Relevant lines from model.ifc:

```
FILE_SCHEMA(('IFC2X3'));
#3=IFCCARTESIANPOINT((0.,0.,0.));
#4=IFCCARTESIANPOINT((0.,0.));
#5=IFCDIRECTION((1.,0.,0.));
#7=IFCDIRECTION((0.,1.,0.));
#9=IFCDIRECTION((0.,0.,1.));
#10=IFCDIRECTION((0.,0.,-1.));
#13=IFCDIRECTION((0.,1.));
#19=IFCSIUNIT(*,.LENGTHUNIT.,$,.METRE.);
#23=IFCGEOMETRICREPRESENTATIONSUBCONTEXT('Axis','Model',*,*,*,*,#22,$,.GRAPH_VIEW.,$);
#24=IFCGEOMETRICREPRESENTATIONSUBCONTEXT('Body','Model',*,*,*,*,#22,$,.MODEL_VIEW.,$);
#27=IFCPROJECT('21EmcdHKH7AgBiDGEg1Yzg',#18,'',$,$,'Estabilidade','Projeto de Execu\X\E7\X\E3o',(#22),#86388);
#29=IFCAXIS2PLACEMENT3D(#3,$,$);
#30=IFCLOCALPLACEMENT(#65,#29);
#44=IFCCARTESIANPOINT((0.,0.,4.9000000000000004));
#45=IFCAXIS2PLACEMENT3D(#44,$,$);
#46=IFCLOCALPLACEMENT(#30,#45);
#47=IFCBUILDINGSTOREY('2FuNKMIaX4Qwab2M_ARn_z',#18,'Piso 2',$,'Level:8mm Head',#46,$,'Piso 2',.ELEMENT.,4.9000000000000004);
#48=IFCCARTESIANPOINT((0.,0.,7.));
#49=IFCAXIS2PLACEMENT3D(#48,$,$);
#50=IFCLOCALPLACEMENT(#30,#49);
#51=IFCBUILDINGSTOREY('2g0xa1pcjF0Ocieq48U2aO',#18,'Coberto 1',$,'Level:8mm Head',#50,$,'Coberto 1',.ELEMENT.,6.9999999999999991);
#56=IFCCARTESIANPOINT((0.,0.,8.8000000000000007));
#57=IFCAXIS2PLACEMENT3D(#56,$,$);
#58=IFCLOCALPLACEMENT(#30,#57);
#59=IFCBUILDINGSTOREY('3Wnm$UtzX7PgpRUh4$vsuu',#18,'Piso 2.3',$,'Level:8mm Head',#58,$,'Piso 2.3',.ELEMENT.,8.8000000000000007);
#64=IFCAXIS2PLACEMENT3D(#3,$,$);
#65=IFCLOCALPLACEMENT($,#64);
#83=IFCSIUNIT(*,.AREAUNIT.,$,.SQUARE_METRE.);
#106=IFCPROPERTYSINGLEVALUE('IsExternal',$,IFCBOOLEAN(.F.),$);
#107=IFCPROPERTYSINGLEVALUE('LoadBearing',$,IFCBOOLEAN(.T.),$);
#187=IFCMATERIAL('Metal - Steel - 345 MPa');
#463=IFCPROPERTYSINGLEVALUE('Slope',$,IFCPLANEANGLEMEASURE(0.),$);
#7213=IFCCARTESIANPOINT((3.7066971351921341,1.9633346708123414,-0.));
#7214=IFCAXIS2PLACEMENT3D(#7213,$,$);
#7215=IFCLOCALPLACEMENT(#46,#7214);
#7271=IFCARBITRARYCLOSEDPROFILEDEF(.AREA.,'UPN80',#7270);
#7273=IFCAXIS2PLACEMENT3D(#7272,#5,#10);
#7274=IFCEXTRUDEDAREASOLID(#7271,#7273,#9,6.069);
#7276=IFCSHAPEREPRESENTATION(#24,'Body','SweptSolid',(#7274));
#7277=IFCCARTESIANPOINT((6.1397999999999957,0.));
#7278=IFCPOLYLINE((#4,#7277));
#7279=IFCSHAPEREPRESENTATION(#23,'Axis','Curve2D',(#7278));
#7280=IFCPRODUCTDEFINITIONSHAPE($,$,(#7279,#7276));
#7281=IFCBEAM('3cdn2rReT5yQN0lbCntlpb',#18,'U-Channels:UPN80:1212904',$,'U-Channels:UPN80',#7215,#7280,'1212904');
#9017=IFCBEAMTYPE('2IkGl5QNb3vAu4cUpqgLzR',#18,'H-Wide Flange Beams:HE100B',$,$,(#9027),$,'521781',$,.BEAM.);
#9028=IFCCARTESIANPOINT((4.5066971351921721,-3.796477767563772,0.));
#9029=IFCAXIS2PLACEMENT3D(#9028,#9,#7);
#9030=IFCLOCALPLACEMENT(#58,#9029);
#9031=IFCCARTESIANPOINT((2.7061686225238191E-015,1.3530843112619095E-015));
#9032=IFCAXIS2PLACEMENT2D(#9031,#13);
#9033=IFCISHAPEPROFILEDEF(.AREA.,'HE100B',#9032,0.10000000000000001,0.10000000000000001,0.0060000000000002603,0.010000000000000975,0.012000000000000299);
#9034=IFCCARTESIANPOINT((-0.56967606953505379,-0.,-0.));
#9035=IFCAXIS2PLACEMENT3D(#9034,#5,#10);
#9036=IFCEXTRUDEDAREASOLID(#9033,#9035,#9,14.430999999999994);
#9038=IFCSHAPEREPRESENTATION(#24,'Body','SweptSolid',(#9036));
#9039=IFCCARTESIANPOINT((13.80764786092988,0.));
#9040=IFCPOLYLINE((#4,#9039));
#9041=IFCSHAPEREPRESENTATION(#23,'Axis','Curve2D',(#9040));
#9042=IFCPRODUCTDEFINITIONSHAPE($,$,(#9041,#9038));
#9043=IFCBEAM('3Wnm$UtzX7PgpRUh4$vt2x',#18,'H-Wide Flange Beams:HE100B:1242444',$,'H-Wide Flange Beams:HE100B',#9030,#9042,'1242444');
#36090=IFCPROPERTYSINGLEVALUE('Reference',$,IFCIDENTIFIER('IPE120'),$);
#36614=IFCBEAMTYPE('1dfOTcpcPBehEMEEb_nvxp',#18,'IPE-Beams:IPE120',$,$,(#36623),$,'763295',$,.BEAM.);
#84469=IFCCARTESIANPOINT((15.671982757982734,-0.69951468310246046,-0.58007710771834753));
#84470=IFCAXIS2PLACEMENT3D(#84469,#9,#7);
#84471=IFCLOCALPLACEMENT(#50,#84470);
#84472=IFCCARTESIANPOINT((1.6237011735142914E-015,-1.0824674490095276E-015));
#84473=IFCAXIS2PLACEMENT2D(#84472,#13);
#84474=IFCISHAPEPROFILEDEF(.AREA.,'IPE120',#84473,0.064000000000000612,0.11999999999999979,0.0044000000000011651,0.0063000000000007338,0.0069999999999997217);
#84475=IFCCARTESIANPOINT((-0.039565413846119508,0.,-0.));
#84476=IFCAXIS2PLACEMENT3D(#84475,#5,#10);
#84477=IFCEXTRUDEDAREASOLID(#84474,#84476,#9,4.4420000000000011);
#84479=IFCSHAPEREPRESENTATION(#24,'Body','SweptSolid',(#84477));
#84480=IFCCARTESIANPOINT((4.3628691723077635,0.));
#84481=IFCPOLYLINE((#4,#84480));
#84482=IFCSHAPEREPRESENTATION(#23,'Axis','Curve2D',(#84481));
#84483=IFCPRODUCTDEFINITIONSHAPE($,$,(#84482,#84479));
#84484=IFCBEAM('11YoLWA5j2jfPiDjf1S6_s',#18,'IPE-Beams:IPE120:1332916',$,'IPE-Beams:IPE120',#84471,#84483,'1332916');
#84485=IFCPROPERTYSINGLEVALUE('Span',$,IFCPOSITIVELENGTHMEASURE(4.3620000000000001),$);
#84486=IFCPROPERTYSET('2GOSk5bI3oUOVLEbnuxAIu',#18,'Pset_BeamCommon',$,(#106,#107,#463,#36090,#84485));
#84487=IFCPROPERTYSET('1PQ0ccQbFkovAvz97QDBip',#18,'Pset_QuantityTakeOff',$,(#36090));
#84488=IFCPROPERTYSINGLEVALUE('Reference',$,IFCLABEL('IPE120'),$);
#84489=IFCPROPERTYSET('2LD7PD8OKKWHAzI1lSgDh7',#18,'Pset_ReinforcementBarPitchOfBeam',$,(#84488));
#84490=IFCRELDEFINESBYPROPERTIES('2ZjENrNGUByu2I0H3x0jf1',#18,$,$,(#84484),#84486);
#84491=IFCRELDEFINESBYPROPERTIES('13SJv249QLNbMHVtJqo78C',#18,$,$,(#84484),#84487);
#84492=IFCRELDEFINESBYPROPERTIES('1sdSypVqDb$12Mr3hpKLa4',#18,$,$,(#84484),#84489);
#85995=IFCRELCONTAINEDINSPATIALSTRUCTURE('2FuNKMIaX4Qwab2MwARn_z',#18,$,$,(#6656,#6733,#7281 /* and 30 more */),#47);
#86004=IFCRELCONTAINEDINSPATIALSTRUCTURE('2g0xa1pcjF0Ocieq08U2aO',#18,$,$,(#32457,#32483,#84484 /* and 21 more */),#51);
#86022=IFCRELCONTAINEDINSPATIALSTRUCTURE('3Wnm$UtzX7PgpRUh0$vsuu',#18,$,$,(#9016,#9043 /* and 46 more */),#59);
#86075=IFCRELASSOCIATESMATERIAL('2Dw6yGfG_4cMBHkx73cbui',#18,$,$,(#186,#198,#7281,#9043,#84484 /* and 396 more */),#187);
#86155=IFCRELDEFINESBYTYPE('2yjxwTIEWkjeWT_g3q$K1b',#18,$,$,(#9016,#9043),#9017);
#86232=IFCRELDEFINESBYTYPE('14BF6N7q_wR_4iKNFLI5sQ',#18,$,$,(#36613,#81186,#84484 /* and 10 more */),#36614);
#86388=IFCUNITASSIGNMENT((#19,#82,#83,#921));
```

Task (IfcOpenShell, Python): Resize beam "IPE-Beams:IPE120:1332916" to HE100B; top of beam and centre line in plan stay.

```python
import ifcopenshell
import ifcopenshell.api.pset
import ifcopenshell.api.type
import ifcopenshell.util.element
import ifcopenshell.util.representation

model = ifcopenshell.open("model.ifc")

member = model.by_id(84484)
source = next(p for p in model.by_type("IfcIShapeProfileDef") if p.ProfileName == "HE100B")

body = ifcopenshell.util.representation.get_representation(member, "Model", "Body")
solid = body.Items[0]
old_profile = solid.SweptArea

# Copy the section's sizes but keep this member's own profile position.
profile = ifcopenshell.util.element.copy(model, source)
# Profiles are centred, so shift by half the change in depth to hold the top.
shift = (old_profile.OverallDepth - profile.OverallDepth) / 2
x, y = old_profile.Position.Location.Coordinates
up = (-1.0, 0.0)  # upwards, in the solid's own plane
location = model.createIfcCartesianPoint((x + up[0] * shift, y + up[1] * shift))
profile.Position = model.createIfcAxis2Placement2D(location, old_profile.Position.RefDirection)
solid.SweptArea = profile
if not model.get_total_inverses(old_profile):
    ifcopenshell.util.element.remove_deep2(model, old_profile)

new_type = model.by_guid("2IkGl5QNb3vAu4cUpqgLzR")
ifcopenshell.api.type.assign_type(
    model, related_objects=[member], relating_type=new_type, should_map_representations=False
)
member.Name = member.Name.replace("IPE120", "HE100B")
member.ObjectType = "IPE-Beams:HE100B"
pset = model.by_id(ifcopenshell.util.element.get_pset(member, "Pset_BeamCommon", should_inherit=False)["id"])
ifcopenshell.api.pset.edit_pset(model, pset=pset, properties={"Reference": "HE100B"})
pset = model.by_id(ifcopenshell.util.element.get_pset(member, "Pset_QuantityTakeOff", should_inherit=False)["id"])
ifcopenshell.api.pset.edit_pset(model, pset=pset, properties={"Reference": "HE100B"})
pset = model.by_id(ifcopenshell.util.element.get_pset(member, "Pset_ReinforcementBarPitchOfBeam", should_inherit=False)["id"])
ifcopenshell.api.pset.edit_pset(model, pset=pset, properties={"Reference": "HE100B"})

print(solid.SweptArea)

model.write("model_v2.ifc")
```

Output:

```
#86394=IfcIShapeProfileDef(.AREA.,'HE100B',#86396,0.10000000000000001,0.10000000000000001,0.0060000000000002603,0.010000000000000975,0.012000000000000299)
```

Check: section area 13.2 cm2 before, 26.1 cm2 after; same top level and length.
